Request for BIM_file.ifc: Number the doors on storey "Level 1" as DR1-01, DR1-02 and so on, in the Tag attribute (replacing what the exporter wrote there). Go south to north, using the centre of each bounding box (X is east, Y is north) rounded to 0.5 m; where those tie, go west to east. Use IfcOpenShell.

First a look at what the model holds.

```python
import ifcopenshell
import ifcopenshell.util.element
import ifcopenshell.util.placement

model = ifcopenshell.open("BIM_file.ifc")
print(model.schema)
storey = next(s for s in model.by_type("IfcBuildingStorey") if s.Name == "Level 1")
doors = [e for e in ifcopenshell.util.element.get_decomposition(storey) if e.is_a("IfcDoor")]
for e in sorted(doors, key=lambda e: e.id()):
    origin = ifcopenshell.util.placement.get_local_placement(e.ObjectPlacement)[:3, 3]
    print(e.id(), e.Tag, e.Name, origin.round(2) + 0.0, sep=" | ")
```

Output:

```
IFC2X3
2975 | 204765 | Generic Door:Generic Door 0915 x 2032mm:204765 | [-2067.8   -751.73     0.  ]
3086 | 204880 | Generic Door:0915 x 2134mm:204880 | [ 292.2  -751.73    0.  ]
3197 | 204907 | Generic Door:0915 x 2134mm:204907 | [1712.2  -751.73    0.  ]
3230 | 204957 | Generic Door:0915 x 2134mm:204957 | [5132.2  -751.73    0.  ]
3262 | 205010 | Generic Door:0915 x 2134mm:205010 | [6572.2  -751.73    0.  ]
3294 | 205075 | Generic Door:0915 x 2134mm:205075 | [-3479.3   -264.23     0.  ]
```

```python
import ifcopenshell
import ifcopenshell.geom
import ifcopenshell.util.element
import ifcopenshell.util.shape

model = ifcopenshell.open("BIM_file.ifc")
settings = ifcopenshell.geom.settings()
settings.set("use-world-coords", True)


def centre(element):
    shape = ifcopenshell.geom.create_shape(settings, element)
    return ifcopenshell.util.shape.get_bbox_centroid(shape.geometry)


storey = next(s for s in model.by_type("IfcBuildingStorey") if s.Name == "Level 1")
doors = [e for e in ifcopenshell.util.element.get_decomposition(storey) if e.is_a("IfcDoor")]

# Insertion points can sit at a corner or the storey origin, so sort by the geometry (in metres).
centres = {e: centre(e) for e in doors}
doors.sort(key=lambda e: (round(centres[e][1] / 0.5), centres[e][0]))

for i, e in enumerate(doors, start=1):
    number = f"DR1-{i:02d}"
    e.Tag = number
    print(e.id(), number)

model.write("BIM_file_v2.ifc")
```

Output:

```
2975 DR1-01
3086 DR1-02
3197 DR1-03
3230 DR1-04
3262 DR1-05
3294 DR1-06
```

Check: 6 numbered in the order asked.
